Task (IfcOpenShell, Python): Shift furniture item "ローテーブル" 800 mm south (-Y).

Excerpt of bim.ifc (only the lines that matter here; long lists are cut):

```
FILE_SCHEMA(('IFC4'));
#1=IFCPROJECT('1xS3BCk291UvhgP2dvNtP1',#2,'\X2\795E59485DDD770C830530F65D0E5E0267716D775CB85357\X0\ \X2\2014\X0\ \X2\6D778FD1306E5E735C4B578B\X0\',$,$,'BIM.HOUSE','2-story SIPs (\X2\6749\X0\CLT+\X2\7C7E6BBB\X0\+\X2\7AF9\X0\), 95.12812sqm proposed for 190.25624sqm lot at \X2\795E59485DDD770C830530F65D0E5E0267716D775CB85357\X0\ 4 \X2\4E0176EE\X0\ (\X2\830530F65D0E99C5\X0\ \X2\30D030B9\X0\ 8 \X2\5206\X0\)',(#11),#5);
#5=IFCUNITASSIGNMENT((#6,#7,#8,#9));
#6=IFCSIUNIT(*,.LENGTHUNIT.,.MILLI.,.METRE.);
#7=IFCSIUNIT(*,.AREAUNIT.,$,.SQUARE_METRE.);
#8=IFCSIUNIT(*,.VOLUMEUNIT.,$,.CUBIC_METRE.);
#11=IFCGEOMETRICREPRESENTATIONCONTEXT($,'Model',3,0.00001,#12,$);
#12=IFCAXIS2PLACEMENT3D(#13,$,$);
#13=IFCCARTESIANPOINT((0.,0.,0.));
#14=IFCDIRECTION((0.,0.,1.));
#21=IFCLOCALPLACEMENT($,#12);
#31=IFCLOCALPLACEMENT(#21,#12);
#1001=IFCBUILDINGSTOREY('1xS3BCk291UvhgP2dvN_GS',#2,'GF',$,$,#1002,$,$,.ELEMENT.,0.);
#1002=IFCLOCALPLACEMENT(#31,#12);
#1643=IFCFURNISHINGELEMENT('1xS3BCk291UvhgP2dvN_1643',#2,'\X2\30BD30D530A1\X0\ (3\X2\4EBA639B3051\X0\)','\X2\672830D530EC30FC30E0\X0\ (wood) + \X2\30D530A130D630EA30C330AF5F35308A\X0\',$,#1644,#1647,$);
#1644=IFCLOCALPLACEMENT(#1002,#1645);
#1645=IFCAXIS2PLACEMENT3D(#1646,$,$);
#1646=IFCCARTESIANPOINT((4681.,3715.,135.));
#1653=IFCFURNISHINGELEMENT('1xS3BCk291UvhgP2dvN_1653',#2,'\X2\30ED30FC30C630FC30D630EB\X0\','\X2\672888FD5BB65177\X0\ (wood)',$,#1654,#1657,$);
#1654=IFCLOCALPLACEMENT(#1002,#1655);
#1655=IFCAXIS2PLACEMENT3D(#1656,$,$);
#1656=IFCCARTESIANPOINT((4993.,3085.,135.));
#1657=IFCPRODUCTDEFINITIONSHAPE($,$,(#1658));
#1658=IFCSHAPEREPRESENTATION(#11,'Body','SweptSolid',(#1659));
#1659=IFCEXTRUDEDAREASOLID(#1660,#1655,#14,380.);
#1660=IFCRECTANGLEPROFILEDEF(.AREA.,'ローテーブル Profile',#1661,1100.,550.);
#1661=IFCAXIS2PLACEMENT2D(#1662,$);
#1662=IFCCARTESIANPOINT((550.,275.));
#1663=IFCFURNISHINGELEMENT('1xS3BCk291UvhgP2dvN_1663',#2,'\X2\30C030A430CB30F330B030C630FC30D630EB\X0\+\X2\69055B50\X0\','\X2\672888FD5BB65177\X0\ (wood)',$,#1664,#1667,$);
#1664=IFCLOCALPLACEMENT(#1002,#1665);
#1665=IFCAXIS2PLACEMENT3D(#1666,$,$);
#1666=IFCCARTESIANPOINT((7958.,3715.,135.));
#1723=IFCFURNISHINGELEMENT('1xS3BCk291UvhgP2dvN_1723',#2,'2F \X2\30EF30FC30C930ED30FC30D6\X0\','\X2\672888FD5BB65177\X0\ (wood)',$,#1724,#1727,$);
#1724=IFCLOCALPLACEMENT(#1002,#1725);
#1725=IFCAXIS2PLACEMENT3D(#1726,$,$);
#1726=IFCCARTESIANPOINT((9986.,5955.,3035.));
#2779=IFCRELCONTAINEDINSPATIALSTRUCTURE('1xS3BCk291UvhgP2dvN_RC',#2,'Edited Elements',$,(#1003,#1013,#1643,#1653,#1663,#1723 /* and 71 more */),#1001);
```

```python
import ifcopenshell
import ifcopenshell.api.geometry
import ifcopenshell.util.placement
import ifcopenshell.util.unit

model = ifcopenshell.open("bim.ifc")
unit_scale = ifcopenshell.util.unit.calculate_unit_scale(model)

item = model.by_guid("1xS3BCk291UvhgP2dvN_1653")
matrix = ifcopenshell.util.placement.get_local_placement(item.ObjectPlacement)
matrix[1, 3] -= 0.8 / unit_scale
ifcopenshell.api.geometry.edit_object_placement(model, product=item, matrix=matrix, is_si=False)

print(ifcopenshell.util.placement.get_local_placement(item.ObjectPlacement).round(3) + 0.0)

model.write("bim_updated.ifc")
```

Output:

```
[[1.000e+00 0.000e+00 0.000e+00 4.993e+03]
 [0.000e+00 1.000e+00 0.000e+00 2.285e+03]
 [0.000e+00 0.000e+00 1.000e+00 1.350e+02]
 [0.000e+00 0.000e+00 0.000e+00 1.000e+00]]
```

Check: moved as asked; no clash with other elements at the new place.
